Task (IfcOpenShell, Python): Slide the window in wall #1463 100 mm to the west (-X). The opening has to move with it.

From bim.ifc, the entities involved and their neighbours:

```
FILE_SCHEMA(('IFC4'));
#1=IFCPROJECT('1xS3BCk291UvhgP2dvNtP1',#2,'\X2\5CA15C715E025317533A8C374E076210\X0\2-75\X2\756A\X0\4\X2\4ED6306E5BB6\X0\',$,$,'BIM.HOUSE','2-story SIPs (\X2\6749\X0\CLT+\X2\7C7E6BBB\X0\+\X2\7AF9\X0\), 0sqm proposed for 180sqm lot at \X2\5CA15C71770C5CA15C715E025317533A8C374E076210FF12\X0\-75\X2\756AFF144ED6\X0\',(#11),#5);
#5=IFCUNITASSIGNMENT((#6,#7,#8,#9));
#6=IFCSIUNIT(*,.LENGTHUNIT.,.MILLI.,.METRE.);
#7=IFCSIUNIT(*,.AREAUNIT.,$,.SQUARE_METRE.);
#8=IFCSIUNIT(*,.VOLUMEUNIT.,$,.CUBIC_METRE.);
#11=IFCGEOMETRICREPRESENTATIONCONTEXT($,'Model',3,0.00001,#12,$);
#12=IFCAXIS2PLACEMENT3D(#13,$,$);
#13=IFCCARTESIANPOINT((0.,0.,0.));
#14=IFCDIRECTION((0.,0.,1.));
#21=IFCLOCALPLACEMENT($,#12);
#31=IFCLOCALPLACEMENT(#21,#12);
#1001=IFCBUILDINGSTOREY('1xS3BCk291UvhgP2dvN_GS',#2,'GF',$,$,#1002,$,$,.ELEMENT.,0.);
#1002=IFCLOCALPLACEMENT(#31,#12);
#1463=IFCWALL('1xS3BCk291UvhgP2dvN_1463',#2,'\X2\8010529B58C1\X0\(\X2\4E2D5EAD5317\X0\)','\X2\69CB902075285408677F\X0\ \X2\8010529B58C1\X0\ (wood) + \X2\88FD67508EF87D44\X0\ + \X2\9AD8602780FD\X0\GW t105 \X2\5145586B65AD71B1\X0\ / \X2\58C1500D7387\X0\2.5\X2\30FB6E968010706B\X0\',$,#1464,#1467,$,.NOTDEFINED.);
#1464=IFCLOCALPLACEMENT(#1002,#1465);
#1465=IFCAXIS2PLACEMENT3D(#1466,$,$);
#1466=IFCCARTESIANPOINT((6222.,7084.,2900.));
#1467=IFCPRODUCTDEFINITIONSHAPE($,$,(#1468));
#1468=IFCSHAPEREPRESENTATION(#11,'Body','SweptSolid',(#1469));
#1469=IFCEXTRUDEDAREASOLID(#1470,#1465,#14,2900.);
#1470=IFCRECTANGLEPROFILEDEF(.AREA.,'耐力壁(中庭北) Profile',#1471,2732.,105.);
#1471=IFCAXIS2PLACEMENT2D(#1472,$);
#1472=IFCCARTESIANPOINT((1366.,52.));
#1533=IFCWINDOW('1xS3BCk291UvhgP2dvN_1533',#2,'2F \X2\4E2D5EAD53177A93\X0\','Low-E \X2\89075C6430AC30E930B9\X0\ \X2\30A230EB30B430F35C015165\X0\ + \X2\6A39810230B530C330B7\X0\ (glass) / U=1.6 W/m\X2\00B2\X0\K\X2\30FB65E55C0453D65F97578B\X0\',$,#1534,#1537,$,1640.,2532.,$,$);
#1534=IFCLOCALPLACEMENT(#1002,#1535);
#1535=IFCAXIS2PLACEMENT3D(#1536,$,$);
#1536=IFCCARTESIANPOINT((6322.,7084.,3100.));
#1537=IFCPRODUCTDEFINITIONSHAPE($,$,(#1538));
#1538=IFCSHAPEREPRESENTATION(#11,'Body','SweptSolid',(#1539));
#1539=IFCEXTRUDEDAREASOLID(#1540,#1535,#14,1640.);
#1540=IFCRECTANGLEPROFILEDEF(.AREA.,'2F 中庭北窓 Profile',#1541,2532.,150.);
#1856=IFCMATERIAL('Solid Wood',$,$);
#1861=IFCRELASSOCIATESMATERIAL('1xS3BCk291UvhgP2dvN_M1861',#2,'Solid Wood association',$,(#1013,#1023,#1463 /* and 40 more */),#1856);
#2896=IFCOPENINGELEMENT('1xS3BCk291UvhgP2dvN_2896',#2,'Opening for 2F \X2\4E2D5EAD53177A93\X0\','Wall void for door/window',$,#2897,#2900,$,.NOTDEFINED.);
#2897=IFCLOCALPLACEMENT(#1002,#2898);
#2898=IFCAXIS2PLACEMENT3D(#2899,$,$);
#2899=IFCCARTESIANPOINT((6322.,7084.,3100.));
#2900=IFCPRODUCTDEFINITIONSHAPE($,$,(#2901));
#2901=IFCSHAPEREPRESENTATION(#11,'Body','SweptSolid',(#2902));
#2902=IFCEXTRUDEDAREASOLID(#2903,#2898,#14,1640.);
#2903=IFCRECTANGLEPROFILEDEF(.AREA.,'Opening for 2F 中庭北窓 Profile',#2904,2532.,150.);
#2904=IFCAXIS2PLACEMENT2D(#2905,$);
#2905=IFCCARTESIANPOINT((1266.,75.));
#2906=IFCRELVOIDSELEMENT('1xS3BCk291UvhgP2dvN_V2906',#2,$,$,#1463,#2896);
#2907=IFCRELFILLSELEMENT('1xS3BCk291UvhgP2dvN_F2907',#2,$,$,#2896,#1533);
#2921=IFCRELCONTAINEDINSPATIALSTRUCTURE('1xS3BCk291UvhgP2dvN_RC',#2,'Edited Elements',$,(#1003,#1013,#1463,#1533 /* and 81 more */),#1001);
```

```python
import ifcopenshell
import ifcopenshell.api.geometry
import ifcopenshell.util.placement
import ifcopenshell.util.unit

model = ifcopenshell.open("bim.ifc")
unit_scale = ifcopenshell.util.unit.calculate_unit_scale(model)

window = model.by_guid("1xS3BCk291UvhgP2dvN_1533")
opening = window.FillsVoids[0].RelatingOpeningElement
wall = opening.VoidsElements[0].RelatingBuildingElement

wall_matrix = ifcopenshell.util.placement.get_local_placement(wall.ObjectPlacement)
shift = wall_matrix[:3, 0] * -0.1 / unit_scale
before = ifcopenshell.util.placement.get_local_placement(window.ObjectPlacement)[:3, 3].copy()

# The window is not placed relative to its opening, so move both.
for product in (opening, window):
    matrix = ifcopenshell.util.placement.get_local_placement(product.ObjectPlacement)
    matrix[:3, 3] += shift
    ifcopenshell.api.geometry.edit_object_placement(model, product=product, matrix=matrix, is_si=False)

after = ifcopenshell.util.placement.get_local_placement(window.ObjectPlacement)[:3, 3]
print("window moved by", (after - before).round(3) + 0.0)

model.write("bim_updated.ifc")
```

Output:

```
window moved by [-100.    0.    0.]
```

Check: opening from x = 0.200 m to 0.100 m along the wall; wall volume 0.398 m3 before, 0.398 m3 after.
